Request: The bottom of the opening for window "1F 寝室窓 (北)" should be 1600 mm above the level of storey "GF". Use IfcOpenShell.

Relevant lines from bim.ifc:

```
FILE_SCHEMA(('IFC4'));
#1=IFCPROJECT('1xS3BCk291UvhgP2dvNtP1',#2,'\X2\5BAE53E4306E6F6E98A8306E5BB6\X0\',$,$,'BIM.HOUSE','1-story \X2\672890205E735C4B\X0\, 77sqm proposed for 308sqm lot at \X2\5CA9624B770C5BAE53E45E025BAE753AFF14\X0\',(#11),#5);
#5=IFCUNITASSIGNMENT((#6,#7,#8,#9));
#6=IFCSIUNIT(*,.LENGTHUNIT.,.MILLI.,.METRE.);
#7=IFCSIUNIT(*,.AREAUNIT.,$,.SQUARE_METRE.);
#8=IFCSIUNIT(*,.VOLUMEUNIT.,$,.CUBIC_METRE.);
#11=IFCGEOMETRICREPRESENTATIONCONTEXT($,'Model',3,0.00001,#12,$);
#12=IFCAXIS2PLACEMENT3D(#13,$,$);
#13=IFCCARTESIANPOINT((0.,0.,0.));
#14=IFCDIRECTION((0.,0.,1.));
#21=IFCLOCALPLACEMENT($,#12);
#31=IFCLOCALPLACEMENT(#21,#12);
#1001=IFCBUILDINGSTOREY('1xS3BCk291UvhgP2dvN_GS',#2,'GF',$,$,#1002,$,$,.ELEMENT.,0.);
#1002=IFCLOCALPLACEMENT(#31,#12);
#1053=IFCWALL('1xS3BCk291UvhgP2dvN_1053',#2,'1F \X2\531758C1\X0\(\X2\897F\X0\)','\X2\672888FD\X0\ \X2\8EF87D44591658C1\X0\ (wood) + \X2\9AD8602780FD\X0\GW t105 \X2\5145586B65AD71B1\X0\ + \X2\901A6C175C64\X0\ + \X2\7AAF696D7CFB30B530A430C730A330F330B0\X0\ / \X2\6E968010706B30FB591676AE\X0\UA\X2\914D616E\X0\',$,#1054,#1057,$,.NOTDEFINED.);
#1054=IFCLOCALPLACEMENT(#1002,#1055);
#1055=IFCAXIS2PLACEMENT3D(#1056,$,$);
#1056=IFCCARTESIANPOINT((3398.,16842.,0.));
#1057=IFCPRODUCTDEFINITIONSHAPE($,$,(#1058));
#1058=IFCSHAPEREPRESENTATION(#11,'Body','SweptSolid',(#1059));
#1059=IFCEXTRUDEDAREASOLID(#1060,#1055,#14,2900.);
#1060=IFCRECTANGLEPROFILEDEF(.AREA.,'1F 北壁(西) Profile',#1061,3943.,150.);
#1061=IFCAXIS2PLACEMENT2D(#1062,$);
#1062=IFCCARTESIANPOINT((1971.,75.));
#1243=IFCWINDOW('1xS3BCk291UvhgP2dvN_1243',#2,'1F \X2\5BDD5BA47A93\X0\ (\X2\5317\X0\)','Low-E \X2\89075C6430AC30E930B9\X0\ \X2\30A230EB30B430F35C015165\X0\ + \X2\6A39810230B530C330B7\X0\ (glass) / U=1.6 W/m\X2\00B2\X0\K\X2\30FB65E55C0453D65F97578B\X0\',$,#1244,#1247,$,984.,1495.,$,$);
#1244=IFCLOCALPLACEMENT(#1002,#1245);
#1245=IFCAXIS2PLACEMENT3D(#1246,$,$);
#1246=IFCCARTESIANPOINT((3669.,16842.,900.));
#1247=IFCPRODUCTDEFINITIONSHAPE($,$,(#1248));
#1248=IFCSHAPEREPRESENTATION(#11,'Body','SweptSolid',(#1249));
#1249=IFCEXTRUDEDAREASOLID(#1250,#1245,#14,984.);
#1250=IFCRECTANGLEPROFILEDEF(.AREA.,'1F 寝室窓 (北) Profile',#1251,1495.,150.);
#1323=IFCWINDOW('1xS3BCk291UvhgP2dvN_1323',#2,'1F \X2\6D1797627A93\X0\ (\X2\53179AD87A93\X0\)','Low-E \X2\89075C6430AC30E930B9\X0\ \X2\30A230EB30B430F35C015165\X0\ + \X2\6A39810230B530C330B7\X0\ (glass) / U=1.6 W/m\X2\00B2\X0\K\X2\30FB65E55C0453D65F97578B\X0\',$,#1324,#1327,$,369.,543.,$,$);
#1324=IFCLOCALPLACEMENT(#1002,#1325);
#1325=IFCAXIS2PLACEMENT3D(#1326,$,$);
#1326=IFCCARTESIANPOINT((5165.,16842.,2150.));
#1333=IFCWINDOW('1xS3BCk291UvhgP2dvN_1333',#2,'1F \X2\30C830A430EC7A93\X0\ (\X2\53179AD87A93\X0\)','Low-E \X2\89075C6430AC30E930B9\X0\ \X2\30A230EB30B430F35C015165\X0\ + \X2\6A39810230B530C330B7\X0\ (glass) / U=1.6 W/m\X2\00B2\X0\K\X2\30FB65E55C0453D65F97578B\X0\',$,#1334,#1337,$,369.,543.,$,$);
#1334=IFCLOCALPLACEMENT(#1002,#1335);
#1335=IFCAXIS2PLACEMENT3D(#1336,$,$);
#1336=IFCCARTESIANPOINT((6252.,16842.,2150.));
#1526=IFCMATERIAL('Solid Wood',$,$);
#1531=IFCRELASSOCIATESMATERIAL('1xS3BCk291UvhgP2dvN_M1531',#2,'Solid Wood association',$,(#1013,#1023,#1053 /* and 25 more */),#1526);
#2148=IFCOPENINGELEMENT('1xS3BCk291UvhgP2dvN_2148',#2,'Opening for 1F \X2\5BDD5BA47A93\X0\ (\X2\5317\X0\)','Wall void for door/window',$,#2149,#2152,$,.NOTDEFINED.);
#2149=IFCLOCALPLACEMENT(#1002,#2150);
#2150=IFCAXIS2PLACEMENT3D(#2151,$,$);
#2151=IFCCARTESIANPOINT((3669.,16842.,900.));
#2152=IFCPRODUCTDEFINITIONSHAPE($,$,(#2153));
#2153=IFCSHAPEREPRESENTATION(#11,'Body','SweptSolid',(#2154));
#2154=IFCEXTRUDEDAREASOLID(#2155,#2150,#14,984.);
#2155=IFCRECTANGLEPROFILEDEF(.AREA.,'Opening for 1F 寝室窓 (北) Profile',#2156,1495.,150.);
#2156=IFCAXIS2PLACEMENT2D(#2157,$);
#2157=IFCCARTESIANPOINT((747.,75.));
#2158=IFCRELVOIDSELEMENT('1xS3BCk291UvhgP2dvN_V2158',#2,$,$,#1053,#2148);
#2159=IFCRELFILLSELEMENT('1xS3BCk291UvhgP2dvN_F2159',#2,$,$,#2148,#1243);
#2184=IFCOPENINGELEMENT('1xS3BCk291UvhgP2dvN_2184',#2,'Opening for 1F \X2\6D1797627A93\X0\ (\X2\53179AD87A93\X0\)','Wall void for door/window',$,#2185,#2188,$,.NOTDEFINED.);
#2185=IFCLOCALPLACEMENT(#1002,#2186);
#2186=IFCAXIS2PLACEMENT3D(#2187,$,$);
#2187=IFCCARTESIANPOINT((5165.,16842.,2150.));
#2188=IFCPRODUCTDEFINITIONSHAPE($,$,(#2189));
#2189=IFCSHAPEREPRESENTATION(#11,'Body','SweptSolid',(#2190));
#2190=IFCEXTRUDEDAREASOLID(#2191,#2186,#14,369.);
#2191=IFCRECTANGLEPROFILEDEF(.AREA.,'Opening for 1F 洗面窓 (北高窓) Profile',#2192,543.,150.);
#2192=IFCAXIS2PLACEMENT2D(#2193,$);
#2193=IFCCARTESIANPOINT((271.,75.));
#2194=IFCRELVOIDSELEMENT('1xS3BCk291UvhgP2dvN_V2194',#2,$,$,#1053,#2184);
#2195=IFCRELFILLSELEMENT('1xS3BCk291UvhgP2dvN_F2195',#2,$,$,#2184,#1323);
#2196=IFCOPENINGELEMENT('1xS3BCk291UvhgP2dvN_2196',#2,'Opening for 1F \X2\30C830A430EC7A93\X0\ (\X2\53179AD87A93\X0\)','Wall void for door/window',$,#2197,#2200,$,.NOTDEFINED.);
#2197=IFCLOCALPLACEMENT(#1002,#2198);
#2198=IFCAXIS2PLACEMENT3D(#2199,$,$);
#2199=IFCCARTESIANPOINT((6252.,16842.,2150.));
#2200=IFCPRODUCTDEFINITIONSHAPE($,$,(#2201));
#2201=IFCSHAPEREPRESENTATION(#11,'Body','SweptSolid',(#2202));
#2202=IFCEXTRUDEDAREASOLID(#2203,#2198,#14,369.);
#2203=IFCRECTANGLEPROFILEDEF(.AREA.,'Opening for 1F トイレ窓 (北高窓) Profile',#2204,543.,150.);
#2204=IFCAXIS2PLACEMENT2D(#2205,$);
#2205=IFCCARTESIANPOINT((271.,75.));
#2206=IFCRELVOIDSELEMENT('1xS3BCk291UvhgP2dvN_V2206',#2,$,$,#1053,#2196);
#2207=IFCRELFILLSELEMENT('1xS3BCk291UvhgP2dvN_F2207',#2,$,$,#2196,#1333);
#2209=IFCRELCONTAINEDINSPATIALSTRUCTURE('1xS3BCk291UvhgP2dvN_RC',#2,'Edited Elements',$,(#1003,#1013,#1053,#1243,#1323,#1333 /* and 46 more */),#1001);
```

```python
import numpy as np
import ifcopenshell
import ifcopenshell.api.geometry
import ifcopenshell.geom
import ifcopenshell.util.element
import ifcopenshell.util.placement
import ifcopenshell.util.shape
import ifcopenshell.util.unit

model = ifcopenshell.open("bim.ifc")
unit_scale = ifcopenshell.util.unit.calculate_unit_scale(model)

window = model.by_id(1243)
opening = window.FillsVoids[0].RelatingOpeningElement
storey = ifcopenshell.util.element.get_container(window, ifc_class="IfcBuildingStorey")
level = ifcopenshell.util.placement.get_local_placement(storey.ObjectPlacement)[2, 3]

# The opening's origin need not be at the sill, so measure its lowest point.
shape = ifcopenshell.geom.create_shape(ifcopenshell.geom.settings(), opening)
bottom = ifcopenshell.util.shape.get_shape_bottom_elevation(shape, shape.geometry) / unit_scale
dz = level + 1600.0 - bottom

shift = np.array([0.0, 0.0, dz])
# The window is not placed relative to its opening, so move both.
for product in (opening, window):
    matrix = ifcopenshell.util.placement.get_local_placement(product.ObjectPlacement)
    matrix[:3, 3] += shift
    ifcopenshell.api.geometry.edit_object_placement(model, product=product, matrix=matrix, is_si=False)

print(f"moved by {dz * unit_scale:+.3f} m")

model.write("bim-out.ifc")
```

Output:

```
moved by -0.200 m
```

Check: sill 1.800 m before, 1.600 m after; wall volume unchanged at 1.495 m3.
